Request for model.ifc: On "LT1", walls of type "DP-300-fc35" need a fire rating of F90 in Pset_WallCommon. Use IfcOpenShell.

First a look at what the model holds.

```python
import ifcopenshell
import ifcopenshell.util.element

model = ifcopenshell.open("model.ifc")
print(model.schema)
storey = next(s for s in model.by_type("IfcBuildingStorey") if s.Name == "LT1")
walls = [e for e in ifcopenshell.util.element.get_decomposition(storey) if e.is_a("IfcWall")]
seen = {}
for e in walls:
    element_type = ifcopenshell.util.element.get_type(e)
    key = (element_type.Name if element_type != e and element_type else None, ifcopenshell.util.element.get_pset(e, "Pset_WallCommon", "FireRating"))
    seen[key] = seen.get(key, 0) + 1
for (name, value), count in sorted(seen.items(), key=str):
    print(count, "x", name, "|", value)
```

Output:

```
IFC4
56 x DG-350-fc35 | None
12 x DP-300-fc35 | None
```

```python
import ifcopenshell
import ifcopenshell.api.pset
import ifcopenshell.util.element

model = ifcopenshell.open("model.ifc")

storey = next(s for s in model.by_type("IfcBuildingStorey") if s.Name == "LT1")
walls = [e for e in ifcopenshell.util.element.get_decomposition(storey) if e.is_a("IfcWall")]

count = 0
for e in walls:
    element_type = ifcopenshell.util.element.get_type(e)
    if element_type in (None, e) or element_type.Name != "DP-300-fc35":
        continue
    # add_pset returns the element's existing set when there is one.
    pset = ifcopenshell.api.pset.add_pset(model, product=e, name="Pset_WallCommon")
    ifcopenshell.api.pset.edit_pset(model, pset=pset, properties={"FireRating": "F90"})
    count += 1

print(count, "walls updated")

model.write("model_rev.ifc")
```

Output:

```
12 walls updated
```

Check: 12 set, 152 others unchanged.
